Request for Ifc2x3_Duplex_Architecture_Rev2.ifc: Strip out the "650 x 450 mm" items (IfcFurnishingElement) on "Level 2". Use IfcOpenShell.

First a look at what the model holds.

```python
import ifcopenshell
import ifcopenshell.util.element

model = ifcopenshell.open("Ifc2x3_Duplex_Architecture_Rev2.ifc")
print(model.schema)
storey = next(s for s in model.by_type("IfcBuildingStorey") if s.Name == "Level 2")
furniture = [e for e in ifcopenshell.util.element.get_decomposition(storey) if e.is_a("IfcFurnishingElement")]
seen = {}
for e in furniture:
    element_type = ifcopenshell.util.element.get_type(e)
    name = element_type.Name if element_type not in (None, e) else None
    seen[name] = seen.get(name, 0) + 1
for name, count in sorted(seen.items(), key=str):
    print(count, "x", name)
```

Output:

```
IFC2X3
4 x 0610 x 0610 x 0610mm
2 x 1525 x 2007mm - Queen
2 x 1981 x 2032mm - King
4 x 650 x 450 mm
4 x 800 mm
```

```python
import ifcopenshell
import ifcopenshell.api.root
import ifcopenshell.util.element

model = ifcopenshell.open("Ifc2x3_Duplex_Architecture_Rev2.ifc")

storey = next(s for s in model.by_type("IfcBuildingStorey") if s.Name == "Level 2")
furniture = [e for e in ifcopenshell.util.element.get_decomposition(storey) if e.is_a("IfcFurnishingElement")]
targets = [e for e in furniture if (t := ifcopenshell.util.element.get_type(e)) not in (None, e) and t.Name == "650 x 450 mm"]

for e in targets:
    ifcopenshell.api.root.remove_product(model, product=e)
print(len(targets), "removed")

model.write("Ifc2x3_Duplex_Architecture_Rev2_updated.ifc")
```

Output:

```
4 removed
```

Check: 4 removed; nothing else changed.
